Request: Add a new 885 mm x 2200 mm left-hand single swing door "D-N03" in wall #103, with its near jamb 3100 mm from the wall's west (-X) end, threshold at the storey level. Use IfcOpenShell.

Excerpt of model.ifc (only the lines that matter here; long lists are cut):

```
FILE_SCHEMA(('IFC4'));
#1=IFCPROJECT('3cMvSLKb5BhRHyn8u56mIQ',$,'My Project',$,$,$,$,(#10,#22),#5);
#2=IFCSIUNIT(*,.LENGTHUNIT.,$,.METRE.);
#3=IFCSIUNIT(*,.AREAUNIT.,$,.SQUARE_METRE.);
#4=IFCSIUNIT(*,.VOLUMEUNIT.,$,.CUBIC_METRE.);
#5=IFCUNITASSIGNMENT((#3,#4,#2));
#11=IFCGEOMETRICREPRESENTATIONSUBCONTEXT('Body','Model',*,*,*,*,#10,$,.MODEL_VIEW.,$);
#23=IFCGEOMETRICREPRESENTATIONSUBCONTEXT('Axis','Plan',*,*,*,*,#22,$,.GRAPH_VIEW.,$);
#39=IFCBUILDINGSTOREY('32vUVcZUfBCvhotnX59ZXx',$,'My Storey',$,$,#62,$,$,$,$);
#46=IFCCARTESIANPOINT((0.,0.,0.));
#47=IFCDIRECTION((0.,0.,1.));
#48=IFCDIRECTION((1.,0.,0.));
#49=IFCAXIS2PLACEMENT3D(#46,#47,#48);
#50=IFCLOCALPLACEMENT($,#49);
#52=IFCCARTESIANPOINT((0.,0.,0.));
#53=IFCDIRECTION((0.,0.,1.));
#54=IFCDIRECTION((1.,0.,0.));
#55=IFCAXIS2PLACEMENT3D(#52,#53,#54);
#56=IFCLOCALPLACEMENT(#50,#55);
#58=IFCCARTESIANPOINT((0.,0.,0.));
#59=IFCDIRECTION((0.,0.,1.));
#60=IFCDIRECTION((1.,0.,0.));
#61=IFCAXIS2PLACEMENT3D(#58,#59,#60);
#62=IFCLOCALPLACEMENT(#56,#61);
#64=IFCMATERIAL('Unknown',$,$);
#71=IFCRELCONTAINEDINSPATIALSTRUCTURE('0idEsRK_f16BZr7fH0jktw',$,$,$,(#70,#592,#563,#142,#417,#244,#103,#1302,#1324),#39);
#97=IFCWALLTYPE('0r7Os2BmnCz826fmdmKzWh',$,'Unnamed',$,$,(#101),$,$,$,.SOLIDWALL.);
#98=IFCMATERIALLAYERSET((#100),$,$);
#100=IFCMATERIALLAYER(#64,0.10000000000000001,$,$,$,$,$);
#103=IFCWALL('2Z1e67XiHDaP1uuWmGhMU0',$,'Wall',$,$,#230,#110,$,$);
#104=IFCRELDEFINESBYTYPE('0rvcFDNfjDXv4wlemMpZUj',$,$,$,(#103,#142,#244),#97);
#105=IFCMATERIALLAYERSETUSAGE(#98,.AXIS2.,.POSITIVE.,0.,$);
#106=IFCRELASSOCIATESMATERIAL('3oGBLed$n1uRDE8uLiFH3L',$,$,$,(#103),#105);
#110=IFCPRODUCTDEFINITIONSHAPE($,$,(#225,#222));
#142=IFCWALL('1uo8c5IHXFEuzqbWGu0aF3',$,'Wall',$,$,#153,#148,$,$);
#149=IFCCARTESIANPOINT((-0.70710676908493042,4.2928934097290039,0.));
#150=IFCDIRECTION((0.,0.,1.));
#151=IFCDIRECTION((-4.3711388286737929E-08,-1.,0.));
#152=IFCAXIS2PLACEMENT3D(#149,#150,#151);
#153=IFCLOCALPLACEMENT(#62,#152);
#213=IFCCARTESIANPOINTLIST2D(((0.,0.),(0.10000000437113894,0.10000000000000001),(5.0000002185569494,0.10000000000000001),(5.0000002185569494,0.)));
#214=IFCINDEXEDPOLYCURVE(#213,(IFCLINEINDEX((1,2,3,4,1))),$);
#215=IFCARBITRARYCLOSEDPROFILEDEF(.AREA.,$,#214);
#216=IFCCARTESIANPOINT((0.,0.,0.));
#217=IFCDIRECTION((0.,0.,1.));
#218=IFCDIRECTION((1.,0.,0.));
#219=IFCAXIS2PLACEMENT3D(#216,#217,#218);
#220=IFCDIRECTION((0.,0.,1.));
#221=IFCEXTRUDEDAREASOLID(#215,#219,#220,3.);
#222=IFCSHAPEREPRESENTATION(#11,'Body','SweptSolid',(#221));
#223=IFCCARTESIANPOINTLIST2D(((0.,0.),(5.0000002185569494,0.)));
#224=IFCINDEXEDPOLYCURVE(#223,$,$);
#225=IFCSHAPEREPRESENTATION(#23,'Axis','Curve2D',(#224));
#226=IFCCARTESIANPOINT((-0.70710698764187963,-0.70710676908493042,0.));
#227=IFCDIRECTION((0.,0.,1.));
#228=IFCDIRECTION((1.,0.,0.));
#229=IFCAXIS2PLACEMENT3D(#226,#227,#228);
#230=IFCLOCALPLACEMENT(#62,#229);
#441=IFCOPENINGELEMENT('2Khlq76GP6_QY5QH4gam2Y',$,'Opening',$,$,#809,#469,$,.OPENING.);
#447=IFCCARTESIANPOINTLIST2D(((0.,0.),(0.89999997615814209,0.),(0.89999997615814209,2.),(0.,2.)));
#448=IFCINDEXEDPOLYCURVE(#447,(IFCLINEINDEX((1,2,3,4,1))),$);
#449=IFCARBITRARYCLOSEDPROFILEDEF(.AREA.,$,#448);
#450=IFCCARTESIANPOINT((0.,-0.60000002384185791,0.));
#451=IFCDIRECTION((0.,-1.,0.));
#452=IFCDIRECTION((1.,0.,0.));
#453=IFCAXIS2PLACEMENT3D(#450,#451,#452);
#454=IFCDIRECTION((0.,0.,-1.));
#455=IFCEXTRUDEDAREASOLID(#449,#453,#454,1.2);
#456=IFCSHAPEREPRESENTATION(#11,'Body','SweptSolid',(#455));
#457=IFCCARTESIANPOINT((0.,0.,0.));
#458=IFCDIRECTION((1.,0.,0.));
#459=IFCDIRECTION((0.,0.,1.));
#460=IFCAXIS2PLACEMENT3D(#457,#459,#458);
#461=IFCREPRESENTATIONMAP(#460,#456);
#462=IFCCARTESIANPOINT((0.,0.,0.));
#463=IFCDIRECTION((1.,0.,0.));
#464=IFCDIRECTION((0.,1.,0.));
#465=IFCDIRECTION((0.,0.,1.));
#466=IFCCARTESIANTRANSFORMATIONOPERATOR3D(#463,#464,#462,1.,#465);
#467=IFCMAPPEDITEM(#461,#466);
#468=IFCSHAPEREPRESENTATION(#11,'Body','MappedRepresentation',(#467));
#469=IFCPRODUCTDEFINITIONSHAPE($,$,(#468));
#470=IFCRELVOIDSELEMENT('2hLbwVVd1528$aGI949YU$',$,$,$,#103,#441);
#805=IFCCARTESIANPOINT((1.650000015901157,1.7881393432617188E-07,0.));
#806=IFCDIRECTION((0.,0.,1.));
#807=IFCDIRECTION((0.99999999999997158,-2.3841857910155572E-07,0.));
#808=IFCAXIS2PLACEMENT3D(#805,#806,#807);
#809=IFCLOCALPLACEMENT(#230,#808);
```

```python
import numpy as np
import ifcopenshell
import ifcopenshell.api.feature
import ifcopenshell.api.geometry
import ifcopenshell.api.root
import ifcopenshell.api.spatial
import ifcopenshell.geom
import ifcopenshell.util.element
import ifcopenshell.util.placement
import ifcopenshell.util.representation
import ifcopenshell.util.shape
import ifcopenshell.util.unit

model = ifcopenshell.open("model.ifc")
unit_scale = ifcopenshell.util.unit.calculate_unit_scale(model)
settings = ifcopenshell.geom.settings()


def volume(element):
    """Net volume in cubic metres, openings subtracted."""
    shape = ifcopenshell.geom.create_shape(settings, element)
    return ifcopenshell.util.shape.get_volume(shape.geometry)


wall = model.by_guid("2Z1e67XiHDaP1uuWmGhMU0")
storey = ifcopenshell.util.element.get_container(wall, ifc_class="IfcBuildingStorey")
context = ifcopenshell.util.representation.get_context(model, "Model", "Body", "MODEL_VIEW")
before = volume(wall)

width, height, from_end, sill = 0.885, 2.2, 3.1, 0.0  # metres

# The wall runs along its own X axis, and the end named is its -X end.
wall_shape = ifcopenshell.geom.create_shape(settings, wall)
x, y, z = ifcopenshell.util.shape.get_vertices(wall_shape.geometry).T
start = x.min() + from_end
face, thickness = float(y.min()), float(y.max() - y.min())
wall_matrix = ifcopenshell.util.placement.get_local_placement(wall.ObjectPlacement)
level = ifcopenshell.util.placement.get_local_placement(storey.ObjectPlacement)[2, 3]


def in_wall(x, y):
    """Placement at x, y metres in the wall's axes, at sill height."""
    matrix = wall_matrix.copy()
    matrix[:, 3] = wall_matrix @ np.array([x / unit_scale, y / unit_scale, 0.0, 1.0])
    matrix[2, 3] = level + sill / unit_scale
    return matrix


# Opening: a box that overshoots both wall faces by 50 mm.
opening = ifcopenshell.api.root.create_entity(model, ifc_class="IfcOpeningElement", predefined_type="OPENING")
box = ifcopenshell.api.geometry.add_wall_representation(
    model, context=context, length=width, height=height, thickness=thickness + 0.1
)
ifcopenshell.api.geometry.assign_representation(model, product=opening, representation=box)
ifcopenshell.api.geometry.edit_object_placement(model, product=opening, matrix=in_wall(start, face - 0.05), is_si=False)
ifcopenshell.api.feature.add_feature(model, feature=opening, element=wall)

door = ifcopenshell.api.root.create_entity(model, ifc_class="IfcDoor", name="D-N03", predefined_type="DOOR")
door.OverallWidth, door.OverallHeight = width / unit_scale, height / unit_scale
door.OperationType = "SINGLE_SWING_LEFT"
body = ifcopenshell.api.geometry.add_door_representation(
    model,
    context=context,
    overall_width=door.OverallWidth,
    overall_height=door.OverallHeight,
    operation_type="SINGLE_SWING_LEFT",
    lining_properties={"LiningDepth": thickness / unit_scale, "ThresholdDepth": thickness / unit_scale},
)
ifcopenshell.api.geometry.assign_representation(model, product=door, representation=body)
ifcopenshell.api.spatial.assign_container(model, products=[door], relating_structure=storey)
ifcopenshell.api.feature.add_filling(model, opening=opening, element=door)

# The lining spans the wall, so the door starts at the wall face.
ifcopenshell.api.geometry.edit_object_placement(model, product=door, matrix=in_wall(start, face), is_si=False)

after = volume(wall)

print(f"wall volume {before:.3f} -> {after:.3f} m3")

model.write("model_v2.ifc")
```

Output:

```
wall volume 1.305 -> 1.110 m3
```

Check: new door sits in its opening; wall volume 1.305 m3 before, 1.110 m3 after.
